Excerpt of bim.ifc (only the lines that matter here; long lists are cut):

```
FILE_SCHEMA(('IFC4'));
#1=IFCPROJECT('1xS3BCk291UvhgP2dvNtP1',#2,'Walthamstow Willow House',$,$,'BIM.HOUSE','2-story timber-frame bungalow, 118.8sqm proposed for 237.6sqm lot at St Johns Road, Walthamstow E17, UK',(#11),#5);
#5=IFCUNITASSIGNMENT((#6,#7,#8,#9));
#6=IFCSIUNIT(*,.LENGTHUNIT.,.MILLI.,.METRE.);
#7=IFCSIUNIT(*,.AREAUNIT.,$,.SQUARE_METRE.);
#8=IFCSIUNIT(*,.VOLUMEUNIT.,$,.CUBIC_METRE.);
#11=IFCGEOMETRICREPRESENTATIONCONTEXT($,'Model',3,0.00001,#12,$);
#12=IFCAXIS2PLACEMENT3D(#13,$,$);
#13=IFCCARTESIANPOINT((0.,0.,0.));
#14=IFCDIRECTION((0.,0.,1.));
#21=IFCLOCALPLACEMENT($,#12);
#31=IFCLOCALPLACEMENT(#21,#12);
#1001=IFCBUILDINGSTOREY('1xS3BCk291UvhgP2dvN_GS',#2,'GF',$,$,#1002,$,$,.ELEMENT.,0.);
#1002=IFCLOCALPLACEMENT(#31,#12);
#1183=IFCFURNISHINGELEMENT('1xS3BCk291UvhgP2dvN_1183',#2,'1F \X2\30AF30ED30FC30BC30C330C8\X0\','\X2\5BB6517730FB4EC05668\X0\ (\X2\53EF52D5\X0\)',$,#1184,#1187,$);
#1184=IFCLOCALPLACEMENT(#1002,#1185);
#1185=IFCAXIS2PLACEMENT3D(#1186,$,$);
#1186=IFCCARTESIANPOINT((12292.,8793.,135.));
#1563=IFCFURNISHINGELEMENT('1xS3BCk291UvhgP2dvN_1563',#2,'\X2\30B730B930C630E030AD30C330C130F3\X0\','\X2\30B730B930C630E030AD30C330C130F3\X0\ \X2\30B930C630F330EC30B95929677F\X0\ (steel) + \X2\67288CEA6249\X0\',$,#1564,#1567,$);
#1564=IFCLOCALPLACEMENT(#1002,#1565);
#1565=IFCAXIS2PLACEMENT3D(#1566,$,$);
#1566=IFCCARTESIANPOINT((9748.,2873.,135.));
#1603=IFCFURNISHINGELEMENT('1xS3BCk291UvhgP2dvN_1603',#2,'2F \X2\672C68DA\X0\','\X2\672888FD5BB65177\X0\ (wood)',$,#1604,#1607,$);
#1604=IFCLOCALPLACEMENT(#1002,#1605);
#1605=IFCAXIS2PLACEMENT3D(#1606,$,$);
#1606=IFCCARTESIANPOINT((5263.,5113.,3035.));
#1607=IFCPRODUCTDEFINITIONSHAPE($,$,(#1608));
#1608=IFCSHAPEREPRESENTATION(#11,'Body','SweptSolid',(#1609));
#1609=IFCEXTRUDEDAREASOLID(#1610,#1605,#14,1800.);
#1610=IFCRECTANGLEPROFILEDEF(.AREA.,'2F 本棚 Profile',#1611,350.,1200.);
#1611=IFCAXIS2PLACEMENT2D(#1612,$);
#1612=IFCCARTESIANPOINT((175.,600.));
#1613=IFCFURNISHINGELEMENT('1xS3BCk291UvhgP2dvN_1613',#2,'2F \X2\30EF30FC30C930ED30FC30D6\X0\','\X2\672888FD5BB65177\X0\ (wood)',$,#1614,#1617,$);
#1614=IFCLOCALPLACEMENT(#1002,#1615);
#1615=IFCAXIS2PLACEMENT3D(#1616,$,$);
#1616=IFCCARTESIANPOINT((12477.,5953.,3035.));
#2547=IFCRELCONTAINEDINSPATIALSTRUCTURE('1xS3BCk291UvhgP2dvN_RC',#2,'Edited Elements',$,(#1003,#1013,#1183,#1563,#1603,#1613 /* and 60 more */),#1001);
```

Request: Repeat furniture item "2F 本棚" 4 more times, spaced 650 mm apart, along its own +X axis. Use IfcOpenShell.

```python
import ifcopenshell
import ifcopenshell.api.geometry
import ifcopenshell.api.root
import ifcopenshell.util.element
import ifcopenshell.util.placement
import ifcopenshell.util.unit

model = ifcopenshell.open("bim.ifc")
unit_scale = ifcopenshell.util.unit.calculate_unit_scale(model)


def reuse_history(source, copy):
    """copy_class also copies each property set's owner history, people and application; keep the originals."""
    for rel in copy.IsDefinedBy:
        if rel.is_a("IfcRelDefinesByProperties") and (history := rel.RelatingPropertyDefinition.OwnerHistory):
            rel.RelatingPropertyDefinition.OwnerHistory = source.OwnerHistory
            ifcopenshell.util.element.remove_deep2(model, history)


source = model.by_id(1603)
base = ifcopenshell.util.placement.get_local_placement(source.ObjectPlacement)
step = base[:3, 0] * 0.65 / unit_scale

for i in range(1, 5):
    copy = ifcopenshell.api.root.copy_class(model, product=source)
    copy.Representation = ifcopenshell.util.element.copy_deep(
        model, source.Representation, exclude=["IfcGeometricRepresentationContext", "IfcRepresentationMap"]
    )
    reuse_history(source, copy)
    matrix = base.copy()
    matrix[:3, 3] += i * step
    print("added at", matrix[:3, 3].round(3) + 0.0)
    ifcopenshell.api.geometry.edit_object_placement(model, product=copy, matrix=matrix, is_si=False)

model.write("bim_rev.ifc")
```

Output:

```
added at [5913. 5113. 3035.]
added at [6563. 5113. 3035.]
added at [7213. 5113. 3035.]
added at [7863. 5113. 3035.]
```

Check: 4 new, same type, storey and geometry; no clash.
